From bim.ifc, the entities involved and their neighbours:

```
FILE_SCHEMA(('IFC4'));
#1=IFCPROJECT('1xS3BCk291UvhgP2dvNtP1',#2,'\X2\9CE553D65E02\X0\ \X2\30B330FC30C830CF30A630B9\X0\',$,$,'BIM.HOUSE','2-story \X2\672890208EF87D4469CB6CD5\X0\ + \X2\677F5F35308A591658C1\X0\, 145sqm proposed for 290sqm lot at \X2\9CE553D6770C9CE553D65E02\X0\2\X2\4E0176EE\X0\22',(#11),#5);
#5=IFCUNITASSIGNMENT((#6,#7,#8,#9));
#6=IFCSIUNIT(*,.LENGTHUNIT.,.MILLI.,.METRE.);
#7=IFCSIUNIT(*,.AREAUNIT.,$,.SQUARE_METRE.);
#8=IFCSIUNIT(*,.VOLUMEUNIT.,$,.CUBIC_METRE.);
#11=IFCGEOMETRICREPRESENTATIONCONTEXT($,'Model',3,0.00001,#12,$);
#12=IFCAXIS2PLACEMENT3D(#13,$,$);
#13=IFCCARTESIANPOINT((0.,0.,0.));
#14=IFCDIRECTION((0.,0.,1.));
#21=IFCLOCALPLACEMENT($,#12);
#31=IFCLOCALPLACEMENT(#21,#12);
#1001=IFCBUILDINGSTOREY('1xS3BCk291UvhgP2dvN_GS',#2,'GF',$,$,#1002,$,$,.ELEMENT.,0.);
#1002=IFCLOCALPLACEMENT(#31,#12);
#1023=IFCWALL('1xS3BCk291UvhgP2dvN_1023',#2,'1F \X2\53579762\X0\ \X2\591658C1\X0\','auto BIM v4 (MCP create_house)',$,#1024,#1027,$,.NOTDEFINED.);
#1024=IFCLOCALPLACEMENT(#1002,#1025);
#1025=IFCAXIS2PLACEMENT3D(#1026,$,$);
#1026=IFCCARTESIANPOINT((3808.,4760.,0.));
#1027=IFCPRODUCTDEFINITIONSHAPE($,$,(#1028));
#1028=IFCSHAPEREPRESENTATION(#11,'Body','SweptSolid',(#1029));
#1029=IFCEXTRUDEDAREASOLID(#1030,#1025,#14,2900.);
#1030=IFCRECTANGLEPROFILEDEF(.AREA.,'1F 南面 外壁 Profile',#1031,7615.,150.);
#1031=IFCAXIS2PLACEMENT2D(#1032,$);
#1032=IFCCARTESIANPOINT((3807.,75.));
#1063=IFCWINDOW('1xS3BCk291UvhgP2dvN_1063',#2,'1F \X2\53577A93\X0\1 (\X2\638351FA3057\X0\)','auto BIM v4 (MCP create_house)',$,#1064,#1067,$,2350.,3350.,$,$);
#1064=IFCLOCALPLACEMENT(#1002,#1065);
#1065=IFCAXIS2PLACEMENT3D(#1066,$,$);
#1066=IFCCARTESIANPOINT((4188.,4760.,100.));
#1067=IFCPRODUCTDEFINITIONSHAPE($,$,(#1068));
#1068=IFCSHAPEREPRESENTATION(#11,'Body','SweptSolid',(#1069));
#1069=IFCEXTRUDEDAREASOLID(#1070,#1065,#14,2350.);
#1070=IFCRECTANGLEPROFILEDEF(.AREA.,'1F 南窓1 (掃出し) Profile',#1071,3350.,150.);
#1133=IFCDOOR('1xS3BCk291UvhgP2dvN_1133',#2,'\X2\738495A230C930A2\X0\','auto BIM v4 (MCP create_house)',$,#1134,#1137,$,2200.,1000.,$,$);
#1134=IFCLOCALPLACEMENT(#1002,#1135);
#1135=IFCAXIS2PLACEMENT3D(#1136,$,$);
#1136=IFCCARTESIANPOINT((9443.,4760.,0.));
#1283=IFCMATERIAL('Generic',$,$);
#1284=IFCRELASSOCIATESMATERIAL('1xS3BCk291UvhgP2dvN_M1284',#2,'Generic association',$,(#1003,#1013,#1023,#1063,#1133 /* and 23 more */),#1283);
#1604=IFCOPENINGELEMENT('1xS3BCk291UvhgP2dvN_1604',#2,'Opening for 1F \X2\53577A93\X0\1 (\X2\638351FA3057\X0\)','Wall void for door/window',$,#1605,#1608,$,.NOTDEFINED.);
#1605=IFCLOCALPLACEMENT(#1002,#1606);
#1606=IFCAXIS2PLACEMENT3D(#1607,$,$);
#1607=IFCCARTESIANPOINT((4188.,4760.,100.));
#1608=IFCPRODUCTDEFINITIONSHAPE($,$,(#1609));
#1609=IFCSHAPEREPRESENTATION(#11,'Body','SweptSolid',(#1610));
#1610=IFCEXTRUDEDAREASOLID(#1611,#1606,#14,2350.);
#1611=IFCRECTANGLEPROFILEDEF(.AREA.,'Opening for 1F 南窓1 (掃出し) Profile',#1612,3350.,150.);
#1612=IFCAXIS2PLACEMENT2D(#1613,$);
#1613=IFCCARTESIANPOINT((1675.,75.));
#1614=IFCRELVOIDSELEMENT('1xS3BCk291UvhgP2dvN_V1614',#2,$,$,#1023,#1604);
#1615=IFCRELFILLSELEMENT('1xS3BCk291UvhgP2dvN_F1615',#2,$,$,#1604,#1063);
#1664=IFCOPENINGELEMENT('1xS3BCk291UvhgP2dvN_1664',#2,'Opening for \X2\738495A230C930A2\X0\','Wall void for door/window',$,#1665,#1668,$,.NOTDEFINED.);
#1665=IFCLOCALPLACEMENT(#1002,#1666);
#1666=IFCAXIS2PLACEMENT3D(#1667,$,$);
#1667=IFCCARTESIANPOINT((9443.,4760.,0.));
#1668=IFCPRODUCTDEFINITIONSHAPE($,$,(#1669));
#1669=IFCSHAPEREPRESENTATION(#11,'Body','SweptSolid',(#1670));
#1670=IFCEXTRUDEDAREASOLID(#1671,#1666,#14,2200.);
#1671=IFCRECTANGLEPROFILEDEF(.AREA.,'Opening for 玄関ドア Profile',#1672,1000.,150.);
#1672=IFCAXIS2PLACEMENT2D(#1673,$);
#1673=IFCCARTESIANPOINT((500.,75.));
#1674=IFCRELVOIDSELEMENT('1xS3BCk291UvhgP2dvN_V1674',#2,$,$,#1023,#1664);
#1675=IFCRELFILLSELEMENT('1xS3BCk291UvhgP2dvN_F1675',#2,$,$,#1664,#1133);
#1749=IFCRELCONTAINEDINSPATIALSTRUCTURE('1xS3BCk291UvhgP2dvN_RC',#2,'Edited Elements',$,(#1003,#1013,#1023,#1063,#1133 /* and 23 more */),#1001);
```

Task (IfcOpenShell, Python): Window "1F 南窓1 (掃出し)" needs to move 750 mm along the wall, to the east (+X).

```python
import ifcopenshell
import ifcopenshell.api.geometry
import ifcopenshell.util.placement
import ifcopenshell.util.unit

model = ifcopenshell.open("bim.ifc")
unit_scale = ifcopenshell.util.unit.calculate_unit_scale(model)

window = model.by_id(1063)
opening = window.FillsVoids[0].RelatingOpeningElement
wall = opening.VoidsElements[0].RelatingBuildingElement

wall_matrix = ifcopenshell.util.placement.get_local_placement(wall.ObjectPlacement)
shift = wall_matrix[:3, 0] * 0.75 / unit_scale
before = ifcopenshell.util.placement.get_local_placement(window.ObjectPlacement)[:3, 3].copy()

# The window is not placed relative to its opening, so move both.
for product in (opening, window):
    matrix = ifcopenshell.util.placement.get_local_placement(product.ObjectPlacement)
    matrix[:3, 3] += shift
    ifcopenshell.api.geometry.edit_object_placement(model, product=product, matrix=matrix, is_si=False)

after = ifcopenshell.util.placement.get_local_placement(window.ObjectPlacement)[:3, 3]
print("window moved by", (after - before).round(3) + 0.0)

model.write("bim_updated.ifc")
```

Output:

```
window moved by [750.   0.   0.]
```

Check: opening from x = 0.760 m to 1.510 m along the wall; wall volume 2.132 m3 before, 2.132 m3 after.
